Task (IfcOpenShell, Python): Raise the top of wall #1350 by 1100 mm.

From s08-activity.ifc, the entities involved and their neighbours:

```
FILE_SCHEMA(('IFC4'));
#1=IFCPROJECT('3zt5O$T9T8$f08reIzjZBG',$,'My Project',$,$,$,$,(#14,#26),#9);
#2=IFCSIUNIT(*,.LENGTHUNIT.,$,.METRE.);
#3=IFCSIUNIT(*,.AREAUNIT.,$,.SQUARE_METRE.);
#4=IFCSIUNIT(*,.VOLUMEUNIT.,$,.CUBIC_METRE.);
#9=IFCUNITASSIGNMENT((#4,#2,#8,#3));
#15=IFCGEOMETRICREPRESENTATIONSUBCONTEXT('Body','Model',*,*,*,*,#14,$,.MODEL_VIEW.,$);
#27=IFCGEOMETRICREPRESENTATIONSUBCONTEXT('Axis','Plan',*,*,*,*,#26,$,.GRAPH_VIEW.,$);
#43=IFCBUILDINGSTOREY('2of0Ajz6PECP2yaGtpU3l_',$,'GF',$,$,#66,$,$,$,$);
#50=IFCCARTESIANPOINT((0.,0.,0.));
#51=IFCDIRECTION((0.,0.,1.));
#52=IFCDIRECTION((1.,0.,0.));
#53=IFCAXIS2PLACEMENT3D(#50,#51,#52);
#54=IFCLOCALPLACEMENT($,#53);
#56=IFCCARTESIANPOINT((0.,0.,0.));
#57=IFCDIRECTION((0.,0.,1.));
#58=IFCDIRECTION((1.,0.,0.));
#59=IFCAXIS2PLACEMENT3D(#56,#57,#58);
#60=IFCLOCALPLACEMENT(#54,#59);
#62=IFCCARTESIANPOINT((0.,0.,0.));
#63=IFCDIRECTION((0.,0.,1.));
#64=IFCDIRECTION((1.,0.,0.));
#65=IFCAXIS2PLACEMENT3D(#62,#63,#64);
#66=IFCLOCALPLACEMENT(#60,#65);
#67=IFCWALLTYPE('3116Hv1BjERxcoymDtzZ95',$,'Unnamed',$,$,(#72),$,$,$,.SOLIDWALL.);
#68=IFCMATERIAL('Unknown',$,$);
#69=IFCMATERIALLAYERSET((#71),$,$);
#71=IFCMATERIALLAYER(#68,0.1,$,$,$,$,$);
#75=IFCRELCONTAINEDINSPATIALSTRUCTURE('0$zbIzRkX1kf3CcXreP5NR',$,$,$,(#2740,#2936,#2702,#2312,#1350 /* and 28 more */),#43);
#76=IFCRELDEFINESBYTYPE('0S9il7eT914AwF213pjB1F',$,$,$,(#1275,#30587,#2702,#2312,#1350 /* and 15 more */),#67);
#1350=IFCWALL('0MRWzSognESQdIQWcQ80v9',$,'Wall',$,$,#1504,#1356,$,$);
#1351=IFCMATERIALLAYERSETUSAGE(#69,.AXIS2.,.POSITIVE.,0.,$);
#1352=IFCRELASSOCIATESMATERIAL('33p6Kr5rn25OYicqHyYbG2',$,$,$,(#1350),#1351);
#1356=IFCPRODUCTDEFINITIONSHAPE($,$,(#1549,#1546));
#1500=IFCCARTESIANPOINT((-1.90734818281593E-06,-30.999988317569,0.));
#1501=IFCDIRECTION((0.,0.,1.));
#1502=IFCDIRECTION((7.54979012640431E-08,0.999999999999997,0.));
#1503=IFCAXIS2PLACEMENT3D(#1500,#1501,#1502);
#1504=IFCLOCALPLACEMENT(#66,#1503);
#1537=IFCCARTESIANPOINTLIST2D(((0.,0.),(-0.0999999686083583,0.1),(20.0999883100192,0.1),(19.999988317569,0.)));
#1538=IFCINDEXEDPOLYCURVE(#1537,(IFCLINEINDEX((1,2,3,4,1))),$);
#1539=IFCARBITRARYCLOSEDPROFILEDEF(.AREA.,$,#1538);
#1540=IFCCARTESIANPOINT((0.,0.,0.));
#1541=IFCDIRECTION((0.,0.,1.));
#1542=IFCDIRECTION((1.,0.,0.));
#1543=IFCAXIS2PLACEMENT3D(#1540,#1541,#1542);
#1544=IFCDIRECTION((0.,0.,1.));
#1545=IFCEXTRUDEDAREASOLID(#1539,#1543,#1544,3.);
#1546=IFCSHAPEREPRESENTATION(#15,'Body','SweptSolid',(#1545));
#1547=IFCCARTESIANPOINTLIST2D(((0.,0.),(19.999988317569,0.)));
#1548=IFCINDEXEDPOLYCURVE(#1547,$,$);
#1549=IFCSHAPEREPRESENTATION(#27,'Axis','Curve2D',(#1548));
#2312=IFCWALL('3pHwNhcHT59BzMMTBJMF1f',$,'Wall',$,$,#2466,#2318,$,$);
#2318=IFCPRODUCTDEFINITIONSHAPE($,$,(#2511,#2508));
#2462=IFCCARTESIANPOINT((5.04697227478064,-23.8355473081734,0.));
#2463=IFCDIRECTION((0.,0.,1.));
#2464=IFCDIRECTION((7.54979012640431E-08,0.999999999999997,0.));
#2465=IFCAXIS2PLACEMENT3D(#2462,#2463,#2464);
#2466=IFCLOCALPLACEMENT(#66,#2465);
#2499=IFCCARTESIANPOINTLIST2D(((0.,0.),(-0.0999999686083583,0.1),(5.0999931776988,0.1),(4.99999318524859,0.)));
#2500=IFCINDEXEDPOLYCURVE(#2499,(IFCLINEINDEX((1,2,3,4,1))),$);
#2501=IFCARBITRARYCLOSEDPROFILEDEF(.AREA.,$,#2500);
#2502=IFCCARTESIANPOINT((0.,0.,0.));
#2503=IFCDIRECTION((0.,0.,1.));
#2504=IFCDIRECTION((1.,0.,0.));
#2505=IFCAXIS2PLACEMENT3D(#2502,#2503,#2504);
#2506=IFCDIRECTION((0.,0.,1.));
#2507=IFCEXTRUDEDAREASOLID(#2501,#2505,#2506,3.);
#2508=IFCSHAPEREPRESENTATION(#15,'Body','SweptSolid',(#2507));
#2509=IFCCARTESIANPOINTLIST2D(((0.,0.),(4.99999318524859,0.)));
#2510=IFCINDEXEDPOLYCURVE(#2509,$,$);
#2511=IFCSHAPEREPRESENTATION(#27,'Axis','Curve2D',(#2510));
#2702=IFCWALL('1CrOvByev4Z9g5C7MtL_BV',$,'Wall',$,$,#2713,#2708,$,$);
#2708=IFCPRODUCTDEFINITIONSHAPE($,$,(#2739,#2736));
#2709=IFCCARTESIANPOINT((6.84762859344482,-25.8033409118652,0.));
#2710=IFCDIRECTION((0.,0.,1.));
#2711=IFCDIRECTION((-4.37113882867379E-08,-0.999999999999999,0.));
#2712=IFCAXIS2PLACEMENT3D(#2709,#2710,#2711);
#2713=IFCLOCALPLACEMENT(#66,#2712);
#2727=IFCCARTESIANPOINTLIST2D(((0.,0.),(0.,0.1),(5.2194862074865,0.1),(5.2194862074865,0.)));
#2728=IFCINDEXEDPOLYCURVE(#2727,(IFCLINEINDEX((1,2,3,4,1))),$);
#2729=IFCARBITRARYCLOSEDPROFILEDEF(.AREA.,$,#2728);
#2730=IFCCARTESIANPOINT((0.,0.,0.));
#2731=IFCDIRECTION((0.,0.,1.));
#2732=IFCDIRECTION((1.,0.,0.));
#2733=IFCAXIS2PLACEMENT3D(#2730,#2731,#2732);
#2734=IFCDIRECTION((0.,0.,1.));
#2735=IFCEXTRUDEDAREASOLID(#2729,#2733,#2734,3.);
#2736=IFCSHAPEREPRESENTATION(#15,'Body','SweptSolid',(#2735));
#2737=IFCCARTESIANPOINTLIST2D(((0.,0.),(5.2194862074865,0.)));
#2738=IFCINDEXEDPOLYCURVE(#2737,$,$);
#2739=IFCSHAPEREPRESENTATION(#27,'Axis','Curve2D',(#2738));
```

```python
import ifcopenshell
import ifcopenshell.geom
import ifcopenshell.util.representation
import ifcopenshell.util.shape
import ifcopenshell.util.unit

model = ifcopenshell.open("s08-activity.ifc")
unit_scale = ifcopenshell.util.unit.calculate_unit_scale(model)
settings = ifcopenshell.geom.settings()


def volume(element):
    """Net volume in cubic metres, openings subtracted."""
    shape = ifcopenshell.geom.create_shape(settings, element)
    return ifcopenshell.util.shape.get_volume(shape.geometry)


wall = model.by_guid("0MRWzSognESQdIQWcQ80v9")
before = volume(wall)

body = ifcopenshell.util.representation.get_representation(wall, "Model", "Body")
solid = body.Items[0]
old_height = solid.Depth
solid.Depth += 1.1 / unit_scale
after = volume(wall)

print(f"height {old_height:g} -> {solid.Depth:g}, volume {before:.3f} -> {after:.3f} m3")

model.write("s08-activity-out.ifc")
```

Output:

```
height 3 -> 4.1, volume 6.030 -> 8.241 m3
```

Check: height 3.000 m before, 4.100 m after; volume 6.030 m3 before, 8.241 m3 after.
